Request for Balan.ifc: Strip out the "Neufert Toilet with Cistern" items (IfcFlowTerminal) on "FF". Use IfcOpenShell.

First a look at what the model holds.

```python
import ifcopenshell
import ifcopenshell.util.element

model = ifcopenshell.open("Balan.ifc")
print(model.schema)
storey = next(s for s in model.by_type("IfcBuildingStorey") if s.Name == "FF")
terminals = [e for e in ifcopenshell.util.element.get_decomposition(storey) if e.is_a("IfcFlowTerminal")]
seen = {}
for e in terminals:
    element_type = ifcopenshell.util.element.get_type(e)
    name = element_type.Name if element_type not in (None, e) else None
    seen[name] = seen.get(name, 0) + 1
for name, count in sorted(seen.items(), key=str):
    print(count, "x", name)
```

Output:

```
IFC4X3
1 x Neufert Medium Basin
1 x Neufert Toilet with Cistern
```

```python
import ifcopenshell
import ifcopenshell.api.root
import ifcopenshell.util.element

model = ifcopenshell.open("Balan.ifc")

storey = next(s for s in model.by_type("IfcBuildingStorey") if s.Name == "FF")
terminals = [e for e in ifcopenshell.util.element.get_decomposition(storey) if e.is_a("IfcFlowTerminal")]
targets = [e for e in terminals if (t := ifcopenshell.util.element.get_type(e)) not in (None, e) and t.Name == "Neufert Toilet with Cistern"]

for e in targets:
    ifcopenshell.api.root.remove_product(model, product=e)
print(len(targets), "removed")

model.write("Balan-out.ifc")
```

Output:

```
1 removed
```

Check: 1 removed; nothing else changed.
